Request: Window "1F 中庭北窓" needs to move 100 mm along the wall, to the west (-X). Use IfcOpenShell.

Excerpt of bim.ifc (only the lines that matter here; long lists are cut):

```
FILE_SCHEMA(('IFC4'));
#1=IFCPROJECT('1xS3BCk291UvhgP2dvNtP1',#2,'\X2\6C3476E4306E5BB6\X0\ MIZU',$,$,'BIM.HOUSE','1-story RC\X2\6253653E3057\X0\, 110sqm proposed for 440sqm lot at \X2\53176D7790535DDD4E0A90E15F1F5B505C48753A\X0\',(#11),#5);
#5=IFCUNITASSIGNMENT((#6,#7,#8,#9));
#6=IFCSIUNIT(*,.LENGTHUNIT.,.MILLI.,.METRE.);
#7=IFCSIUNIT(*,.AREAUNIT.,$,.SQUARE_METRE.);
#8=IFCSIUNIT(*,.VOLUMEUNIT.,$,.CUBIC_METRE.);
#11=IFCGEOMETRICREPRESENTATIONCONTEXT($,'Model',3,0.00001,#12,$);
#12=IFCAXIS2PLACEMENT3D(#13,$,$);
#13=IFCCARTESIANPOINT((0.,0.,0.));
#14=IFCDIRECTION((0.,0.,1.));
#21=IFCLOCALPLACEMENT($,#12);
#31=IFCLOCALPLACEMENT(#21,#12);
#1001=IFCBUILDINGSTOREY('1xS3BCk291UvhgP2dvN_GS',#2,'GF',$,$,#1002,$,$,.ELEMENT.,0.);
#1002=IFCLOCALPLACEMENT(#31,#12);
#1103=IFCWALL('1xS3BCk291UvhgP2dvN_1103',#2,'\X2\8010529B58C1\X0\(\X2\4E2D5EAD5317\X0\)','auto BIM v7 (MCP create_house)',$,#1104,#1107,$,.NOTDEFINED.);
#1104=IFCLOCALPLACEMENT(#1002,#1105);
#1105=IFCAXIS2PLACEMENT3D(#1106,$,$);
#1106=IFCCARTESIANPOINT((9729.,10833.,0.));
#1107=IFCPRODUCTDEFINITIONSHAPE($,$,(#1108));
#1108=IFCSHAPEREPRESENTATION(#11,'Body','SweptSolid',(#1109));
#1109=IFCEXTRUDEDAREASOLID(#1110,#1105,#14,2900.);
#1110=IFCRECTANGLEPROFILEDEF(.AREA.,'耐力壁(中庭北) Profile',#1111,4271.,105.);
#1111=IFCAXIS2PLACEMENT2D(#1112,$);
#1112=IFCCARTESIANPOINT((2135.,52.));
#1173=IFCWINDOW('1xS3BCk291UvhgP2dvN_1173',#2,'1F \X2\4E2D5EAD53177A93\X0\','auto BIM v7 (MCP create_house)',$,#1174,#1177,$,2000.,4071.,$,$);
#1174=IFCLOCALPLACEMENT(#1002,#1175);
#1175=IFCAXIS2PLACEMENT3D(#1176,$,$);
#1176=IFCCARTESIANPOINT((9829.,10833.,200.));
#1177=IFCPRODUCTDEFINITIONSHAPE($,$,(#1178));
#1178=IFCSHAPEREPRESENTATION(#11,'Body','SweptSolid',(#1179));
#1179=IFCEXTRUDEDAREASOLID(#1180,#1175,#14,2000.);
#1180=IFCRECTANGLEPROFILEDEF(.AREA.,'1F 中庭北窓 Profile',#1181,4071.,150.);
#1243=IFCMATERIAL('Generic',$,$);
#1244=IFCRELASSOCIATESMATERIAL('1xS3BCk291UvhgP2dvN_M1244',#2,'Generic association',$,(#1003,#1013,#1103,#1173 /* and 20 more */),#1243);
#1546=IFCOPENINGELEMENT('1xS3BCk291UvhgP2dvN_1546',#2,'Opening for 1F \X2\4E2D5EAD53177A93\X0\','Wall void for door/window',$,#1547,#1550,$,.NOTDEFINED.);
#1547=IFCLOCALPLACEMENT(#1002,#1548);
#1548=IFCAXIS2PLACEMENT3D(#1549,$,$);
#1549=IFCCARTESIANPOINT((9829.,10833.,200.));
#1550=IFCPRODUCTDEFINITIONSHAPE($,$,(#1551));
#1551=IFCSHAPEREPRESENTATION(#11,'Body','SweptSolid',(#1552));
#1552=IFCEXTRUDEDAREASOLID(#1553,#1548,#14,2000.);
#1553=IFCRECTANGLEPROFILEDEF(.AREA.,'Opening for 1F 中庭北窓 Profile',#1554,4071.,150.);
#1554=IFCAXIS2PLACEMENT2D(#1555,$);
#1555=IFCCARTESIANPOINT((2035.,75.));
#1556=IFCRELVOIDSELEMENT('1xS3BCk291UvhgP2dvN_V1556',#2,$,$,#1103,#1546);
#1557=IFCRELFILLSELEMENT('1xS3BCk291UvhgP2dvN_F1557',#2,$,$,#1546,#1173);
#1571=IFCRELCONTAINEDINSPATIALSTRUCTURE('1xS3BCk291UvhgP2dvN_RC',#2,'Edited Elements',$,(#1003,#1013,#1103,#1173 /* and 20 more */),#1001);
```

```python
import ifcopenshell
import ifcopenshell.api.geometry
import ifcopenshell.util.placement

model = ifcopenshell.open("bim.ifc")

window = model.by_guid("1xS3BCk291UvhgP2dvN_1173")
opening = window.FillsVoids[0].RelatingOpeningElement
wall = opening.VoidsElements[0].RelatingBuildingElement

wall_matrix = ifcopenshell.util.placement.get_local_placement(wall.ObjectPlacement)
shift = wall_matrix[:3, 0] * -100.0
before = ifcopenshell.util.placement.get_local_placement(window.ObjectPlacement)[:3, 3].copy()

# The window is not placed relative to its opening, so move both.
for product in (opening, window):
    matrix = ifcopenshell.util.placement.get_local_placement(product.ObjectPlacement)
    matrix[:3, 3] += shift
    ifcopenshell.api.geometry.edit_object_placement(model, product=product, matrix=matrix, is_si=False)

after = ifcopenshell.util.placement.get_local_placement(window.ObjectPlacement)[:3, 3]
print("window moved by", (after - before).round(3) + 0.0)

model.write("bim_updated.ifc")
```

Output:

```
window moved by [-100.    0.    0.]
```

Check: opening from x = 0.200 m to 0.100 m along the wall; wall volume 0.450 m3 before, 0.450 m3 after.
